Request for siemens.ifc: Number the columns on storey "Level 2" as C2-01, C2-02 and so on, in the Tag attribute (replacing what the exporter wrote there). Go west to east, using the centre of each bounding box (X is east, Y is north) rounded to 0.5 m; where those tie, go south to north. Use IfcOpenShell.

First a look at what the model holds.

```python
import ifcopenshell
import ifcopenshell.util.element
import ifcopenshell.util.placement

model = ifcopenshell.open("siemens.ifc")
print(model.schema)
storey = next(s for s in model.by_type("IfcBuildingStorey") if s.Name == "Level 2")
columns = [e for e in ifcopenshell.util.element.get_decomposition(storey) if e.is_a("IfcColumn")]
for e in sorted(columns, key=lambda e: e.id()):
    origin = ifcopenshell.util.placement.get_local_placement(e.ObjectPlacement)[:3, 3]
    print(e.id(), e.Tag, e.Name, origin.round(2) + 0.0, sep=" | ")
```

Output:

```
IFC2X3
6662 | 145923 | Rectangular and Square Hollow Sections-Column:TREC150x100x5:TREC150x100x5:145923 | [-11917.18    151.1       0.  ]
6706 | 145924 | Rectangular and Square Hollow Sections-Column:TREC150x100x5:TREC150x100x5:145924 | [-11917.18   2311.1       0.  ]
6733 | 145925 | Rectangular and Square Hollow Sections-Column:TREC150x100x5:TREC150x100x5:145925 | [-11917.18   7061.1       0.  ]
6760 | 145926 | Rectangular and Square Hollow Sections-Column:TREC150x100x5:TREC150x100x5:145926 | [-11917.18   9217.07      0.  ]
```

```python
import ifcopenshell
import ifcopenshell.geom
import ifcopenshell.util.element
import ifcopenshell.util.shape

model = ifcopenshell.open("siemens.ifc")
settings = ifcopenshell.geom.settings()
settings.set("use-world-coords", True)


def centre(element):
    shape = ifcopenshell.geom.create_shape(settings, element)
    return ifcopenshell.util.shape.get_bbox_centroid(shape.geometry)


storey = next(s for s in model.by_type("IfcBuildingStorey") if s.Name == "Level 2")
columns = [e for e in ifcopenshell.util.element.get_decomposition(storey) if e.is_a("IfcColumn")]

# Insertion points can sit at a corner or the storey origin, so sort by the geometry (in metres).
centres = {e: centre(e) for e in columns}
columns.sort(key=lambda e: (round(centres[e][0] / 0.5), centres[e][1]))

for i, e in enumerate(columns, start=1):
    number = f"C2-{i:02d}"
    e.Tag = number
    print(e.id(), number)

model.write("siemens_rev.ifc")
```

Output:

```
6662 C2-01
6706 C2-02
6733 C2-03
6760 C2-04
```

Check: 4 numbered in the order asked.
